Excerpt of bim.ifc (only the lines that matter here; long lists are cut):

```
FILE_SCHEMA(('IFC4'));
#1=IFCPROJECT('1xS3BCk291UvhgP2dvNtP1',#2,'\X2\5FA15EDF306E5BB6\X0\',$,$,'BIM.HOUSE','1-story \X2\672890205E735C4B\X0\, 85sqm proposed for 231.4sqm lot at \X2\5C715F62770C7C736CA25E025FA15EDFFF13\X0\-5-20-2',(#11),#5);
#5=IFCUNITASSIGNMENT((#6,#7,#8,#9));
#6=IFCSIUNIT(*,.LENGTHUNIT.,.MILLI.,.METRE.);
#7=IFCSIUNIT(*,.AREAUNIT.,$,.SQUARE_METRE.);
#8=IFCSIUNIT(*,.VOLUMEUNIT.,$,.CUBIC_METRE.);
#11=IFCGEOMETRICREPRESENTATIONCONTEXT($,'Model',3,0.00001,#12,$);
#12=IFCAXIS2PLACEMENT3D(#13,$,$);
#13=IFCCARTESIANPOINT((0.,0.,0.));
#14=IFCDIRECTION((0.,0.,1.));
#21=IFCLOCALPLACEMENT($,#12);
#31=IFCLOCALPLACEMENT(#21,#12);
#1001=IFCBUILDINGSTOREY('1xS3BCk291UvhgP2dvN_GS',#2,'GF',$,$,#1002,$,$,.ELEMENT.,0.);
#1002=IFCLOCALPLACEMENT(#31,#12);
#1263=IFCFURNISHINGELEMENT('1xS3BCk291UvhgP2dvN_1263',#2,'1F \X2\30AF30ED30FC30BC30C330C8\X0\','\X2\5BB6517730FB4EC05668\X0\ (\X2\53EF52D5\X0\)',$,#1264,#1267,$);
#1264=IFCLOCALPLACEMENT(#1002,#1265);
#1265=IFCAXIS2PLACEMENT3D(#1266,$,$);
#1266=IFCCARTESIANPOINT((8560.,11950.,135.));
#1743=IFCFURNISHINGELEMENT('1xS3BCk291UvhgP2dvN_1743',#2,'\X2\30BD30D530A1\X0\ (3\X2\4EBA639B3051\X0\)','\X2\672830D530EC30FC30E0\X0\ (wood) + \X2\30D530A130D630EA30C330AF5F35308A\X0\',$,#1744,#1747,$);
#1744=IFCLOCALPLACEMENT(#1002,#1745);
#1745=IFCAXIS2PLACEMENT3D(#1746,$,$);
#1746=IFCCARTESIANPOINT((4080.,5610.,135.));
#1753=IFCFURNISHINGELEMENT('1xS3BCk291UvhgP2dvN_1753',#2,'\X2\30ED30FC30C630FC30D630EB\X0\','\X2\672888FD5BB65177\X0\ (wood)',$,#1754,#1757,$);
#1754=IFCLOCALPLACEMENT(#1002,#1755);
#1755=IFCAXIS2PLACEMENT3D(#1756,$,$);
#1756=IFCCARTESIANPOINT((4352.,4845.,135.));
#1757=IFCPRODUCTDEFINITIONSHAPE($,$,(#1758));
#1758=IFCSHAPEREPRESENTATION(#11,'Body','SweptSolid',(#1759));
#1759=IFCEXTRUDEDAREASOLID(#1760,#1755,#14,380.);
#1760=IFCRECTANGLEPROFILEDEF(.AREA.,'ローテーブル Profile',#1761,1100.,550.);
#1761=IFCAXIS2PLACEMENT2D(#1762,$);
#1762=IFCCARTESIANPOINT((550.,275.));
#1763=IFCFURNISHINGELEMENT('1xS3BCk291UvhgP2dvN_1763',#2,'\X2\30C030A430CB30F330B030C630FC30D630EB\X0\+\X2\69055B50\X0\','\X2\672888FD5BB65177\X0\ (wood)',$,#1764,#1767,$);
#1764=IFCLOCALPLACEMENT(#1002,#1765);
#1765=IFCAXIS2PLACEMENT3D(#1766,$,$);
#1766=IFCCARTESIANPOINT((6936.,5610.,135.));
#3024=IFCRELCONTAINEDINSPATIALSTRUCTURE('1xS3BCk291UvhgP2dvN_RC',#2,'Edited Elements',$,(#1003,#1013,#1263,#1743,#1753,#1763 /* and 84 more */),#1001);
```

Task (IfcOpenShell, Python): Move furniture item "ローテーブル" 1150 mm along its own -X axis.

```python
import ifcopenshell
import ifcopenshell.api.geometry
import ifcopenshell.util.placement
import ifcopenshell.util.unit

model = ifcopenshell.open("bim.ifc")
unit_scale = ifcopenshell.util.unit.calculate_unit_scale(model)

item = model.by_guid("1xS3BCk291UvhgP2dvN_1753")
matrix = ifcopenshell.util.placement.get_local_placement(item.ObjectPlacement)
matrix[:3, 3] -= matrix[:3, 0] * 1.15 / unit_scale
ifcopenshell.api.geometry.edit_object_placement(model, product=item, matrix=matrix, is_si=False)

print(ifcopenshell.util.placement.get_local_placement(item.ObjectPlacement).round(3) + 0.0)

model.write("bim_rev.ifc")
```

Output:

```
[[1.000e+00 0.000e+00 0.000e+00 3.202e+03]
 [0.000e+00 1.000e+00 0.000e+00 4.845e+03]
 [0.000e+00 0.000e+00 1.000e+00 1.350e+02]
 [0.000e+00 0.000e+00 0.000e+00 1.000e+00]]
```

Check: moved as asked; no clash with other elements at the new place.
